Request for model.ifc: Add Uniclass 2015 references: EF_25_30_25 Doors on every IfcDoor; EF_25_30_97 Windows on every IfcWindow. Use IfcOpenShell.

First a look at what the model holds.

```python
import ifcopenshell

model = ifcopenshell.open("model.ifc")
print(model.schema)
print("classifications:", [c.Name for c in model.by_type("IfcClassification")])
for ifc_class in ("IfcDoor", "IfcRoof", "IfcStair", "IfcWall", "IfcWindow"):
    print(ifc_class, len(model.by_type(ifc_class)))
```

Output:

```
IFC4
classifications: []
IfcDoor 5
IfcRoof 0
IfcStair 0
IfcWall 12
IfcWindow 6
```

```python
import ifcopenshell
import ifcopenshell.api.classification

model = ifcopenshell.open("model.ifc")

system = ifcopenshell.api.classification.add_classification(model, classification="Uniclass 2015")

codes = {
    "IfcDoor": ("EF_25_30_25", "Doors"),
    "IfcWindow": ("EF_25_30_97", "Windows"),
}
for ifc_class, (code, name) in codes.items():
    products = model.by_type(ifc_class)
    ifcopenshell.api.classification.add_reference(
        model, products=products, classification=system, identification=code, name=name
    )
    print(code, len(products))

model.write("model-out.ifc")
```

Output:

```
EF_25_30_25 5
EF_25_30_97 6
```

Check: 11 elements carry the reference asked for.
